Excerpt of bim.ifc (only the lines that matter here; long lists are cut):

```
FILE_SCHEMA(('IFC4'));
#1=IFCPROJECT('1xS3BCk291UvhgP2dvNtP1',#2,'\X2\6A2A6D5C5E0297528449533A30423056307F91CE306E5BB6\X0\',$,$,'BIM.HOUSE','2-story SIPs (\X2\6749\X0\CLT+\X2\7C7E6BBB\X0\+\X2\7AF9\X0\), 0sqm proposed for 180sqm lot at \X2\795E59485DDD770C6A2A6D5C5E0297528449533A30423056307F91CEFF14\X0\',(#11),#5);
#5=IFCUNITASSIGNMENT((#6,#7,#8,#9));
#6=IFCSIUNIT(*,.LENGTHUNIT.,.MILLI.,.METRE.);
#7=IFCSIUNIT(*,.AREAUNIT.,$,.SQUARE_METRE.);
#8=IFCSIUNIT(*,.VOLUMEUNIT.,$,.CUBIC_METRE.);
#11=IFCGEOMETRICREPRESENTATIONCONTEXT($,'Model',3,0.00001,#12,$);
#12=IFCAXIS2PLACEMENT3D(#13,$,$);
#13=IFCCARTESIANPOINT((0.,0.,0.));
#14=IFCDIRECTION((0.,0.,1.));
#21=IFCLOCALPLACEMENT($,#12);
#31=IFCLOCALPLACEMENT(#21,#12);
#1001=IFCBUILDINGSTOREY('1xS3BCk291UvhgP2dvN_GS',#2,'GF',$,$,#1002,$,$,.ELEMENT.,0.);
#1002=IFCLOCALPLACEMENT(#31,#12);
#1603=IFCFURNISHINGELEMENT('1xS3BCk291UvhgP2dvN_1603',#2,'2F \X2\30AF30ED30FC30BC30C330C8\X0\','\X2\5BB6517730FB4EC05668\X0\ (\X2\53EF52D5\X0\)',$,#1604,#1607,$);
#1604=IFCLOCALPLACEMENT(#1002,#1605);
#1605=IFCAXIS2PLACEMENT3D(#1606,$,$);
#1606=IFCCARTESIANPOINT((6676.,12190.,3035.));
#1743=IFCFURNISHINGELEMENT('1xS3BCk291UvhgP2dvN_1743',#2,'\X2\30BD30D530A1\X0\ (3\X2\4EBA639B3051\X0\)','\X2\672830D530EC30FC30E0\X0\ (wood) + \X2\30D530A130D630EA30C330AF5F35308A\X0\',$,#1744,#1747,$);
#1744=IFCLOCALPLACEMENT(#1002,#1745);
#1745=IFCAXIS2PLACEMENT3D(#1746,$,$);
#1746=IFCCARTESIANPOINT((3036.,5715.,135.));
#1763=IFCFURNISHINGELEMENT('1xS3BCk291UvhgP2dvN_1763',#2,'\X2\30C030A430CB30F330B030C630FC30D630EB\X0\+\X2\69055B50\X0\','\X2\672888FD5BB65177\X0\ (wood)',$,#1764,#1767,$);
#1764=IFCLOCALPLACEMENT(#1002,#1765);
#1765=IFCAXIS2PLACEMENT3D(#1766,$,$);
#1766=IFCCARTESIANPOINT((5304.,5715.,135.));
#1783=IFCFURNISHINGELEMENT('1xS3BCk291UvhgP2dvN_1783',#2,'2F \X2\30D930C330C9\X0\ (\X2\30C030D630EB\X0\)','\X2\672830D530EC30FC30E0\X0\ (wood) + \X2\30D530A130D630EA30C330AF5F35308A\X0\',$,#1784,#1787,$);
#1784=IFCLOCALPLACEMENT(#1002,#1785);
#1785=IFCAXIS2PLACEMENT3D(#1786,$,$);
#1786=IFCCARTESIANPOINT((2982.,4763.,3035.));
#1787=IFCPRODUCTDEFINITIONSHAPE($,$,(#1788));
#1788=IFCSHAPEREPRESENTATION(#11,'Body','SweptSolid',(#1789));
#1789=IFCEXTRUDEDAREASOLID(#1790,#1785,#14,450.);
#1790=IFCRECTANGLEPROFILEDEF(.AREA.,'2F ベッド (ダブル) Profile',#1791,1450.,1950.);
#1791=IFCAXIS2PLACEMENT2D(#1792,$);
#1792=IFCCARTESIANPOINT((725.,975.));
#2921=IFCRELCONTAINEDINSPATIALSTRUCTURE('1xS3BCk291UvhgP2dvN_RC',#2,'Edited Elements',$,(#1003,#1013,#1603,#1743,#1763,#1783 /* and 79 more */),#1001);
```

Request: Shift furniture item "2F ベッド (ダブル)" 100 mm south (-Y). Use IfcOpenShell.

```python
import ifcopenshell
import ifcopenshell.api.geometry
import ifcopenshell.util.placement
import ifcopenshell.util.unit

model = ifcopenshell.open("bim.ifc")
unit_scale = ifcopenshell.util.unit.calculate_unit_scale(model)

item = model.by_guid("1xS3BCk291UvhgP2dvN_1783")
matrix = ifcopenshell.util.placement.get_local_placement(item.ObjectPlacement)
matrix[1, 3] -= 0.1 / unit_scale
ifcopenshell.api.geometry.edit_object_placement(model, product=item, matrix=matrix, is_si=False)

print(ifcopenshell.util.placement.get_local_placement(item.ObjectPlacement).round(3) + 0.0)

model.write("bim_rev.ifc")
```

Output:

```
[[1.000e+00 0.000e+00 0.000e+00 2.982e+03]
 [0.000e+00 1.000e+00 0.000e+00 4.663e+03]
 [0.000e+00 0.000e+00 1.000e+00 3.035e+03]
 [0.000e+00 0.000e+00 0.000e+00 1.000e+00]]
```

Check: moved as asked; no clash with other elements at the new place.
